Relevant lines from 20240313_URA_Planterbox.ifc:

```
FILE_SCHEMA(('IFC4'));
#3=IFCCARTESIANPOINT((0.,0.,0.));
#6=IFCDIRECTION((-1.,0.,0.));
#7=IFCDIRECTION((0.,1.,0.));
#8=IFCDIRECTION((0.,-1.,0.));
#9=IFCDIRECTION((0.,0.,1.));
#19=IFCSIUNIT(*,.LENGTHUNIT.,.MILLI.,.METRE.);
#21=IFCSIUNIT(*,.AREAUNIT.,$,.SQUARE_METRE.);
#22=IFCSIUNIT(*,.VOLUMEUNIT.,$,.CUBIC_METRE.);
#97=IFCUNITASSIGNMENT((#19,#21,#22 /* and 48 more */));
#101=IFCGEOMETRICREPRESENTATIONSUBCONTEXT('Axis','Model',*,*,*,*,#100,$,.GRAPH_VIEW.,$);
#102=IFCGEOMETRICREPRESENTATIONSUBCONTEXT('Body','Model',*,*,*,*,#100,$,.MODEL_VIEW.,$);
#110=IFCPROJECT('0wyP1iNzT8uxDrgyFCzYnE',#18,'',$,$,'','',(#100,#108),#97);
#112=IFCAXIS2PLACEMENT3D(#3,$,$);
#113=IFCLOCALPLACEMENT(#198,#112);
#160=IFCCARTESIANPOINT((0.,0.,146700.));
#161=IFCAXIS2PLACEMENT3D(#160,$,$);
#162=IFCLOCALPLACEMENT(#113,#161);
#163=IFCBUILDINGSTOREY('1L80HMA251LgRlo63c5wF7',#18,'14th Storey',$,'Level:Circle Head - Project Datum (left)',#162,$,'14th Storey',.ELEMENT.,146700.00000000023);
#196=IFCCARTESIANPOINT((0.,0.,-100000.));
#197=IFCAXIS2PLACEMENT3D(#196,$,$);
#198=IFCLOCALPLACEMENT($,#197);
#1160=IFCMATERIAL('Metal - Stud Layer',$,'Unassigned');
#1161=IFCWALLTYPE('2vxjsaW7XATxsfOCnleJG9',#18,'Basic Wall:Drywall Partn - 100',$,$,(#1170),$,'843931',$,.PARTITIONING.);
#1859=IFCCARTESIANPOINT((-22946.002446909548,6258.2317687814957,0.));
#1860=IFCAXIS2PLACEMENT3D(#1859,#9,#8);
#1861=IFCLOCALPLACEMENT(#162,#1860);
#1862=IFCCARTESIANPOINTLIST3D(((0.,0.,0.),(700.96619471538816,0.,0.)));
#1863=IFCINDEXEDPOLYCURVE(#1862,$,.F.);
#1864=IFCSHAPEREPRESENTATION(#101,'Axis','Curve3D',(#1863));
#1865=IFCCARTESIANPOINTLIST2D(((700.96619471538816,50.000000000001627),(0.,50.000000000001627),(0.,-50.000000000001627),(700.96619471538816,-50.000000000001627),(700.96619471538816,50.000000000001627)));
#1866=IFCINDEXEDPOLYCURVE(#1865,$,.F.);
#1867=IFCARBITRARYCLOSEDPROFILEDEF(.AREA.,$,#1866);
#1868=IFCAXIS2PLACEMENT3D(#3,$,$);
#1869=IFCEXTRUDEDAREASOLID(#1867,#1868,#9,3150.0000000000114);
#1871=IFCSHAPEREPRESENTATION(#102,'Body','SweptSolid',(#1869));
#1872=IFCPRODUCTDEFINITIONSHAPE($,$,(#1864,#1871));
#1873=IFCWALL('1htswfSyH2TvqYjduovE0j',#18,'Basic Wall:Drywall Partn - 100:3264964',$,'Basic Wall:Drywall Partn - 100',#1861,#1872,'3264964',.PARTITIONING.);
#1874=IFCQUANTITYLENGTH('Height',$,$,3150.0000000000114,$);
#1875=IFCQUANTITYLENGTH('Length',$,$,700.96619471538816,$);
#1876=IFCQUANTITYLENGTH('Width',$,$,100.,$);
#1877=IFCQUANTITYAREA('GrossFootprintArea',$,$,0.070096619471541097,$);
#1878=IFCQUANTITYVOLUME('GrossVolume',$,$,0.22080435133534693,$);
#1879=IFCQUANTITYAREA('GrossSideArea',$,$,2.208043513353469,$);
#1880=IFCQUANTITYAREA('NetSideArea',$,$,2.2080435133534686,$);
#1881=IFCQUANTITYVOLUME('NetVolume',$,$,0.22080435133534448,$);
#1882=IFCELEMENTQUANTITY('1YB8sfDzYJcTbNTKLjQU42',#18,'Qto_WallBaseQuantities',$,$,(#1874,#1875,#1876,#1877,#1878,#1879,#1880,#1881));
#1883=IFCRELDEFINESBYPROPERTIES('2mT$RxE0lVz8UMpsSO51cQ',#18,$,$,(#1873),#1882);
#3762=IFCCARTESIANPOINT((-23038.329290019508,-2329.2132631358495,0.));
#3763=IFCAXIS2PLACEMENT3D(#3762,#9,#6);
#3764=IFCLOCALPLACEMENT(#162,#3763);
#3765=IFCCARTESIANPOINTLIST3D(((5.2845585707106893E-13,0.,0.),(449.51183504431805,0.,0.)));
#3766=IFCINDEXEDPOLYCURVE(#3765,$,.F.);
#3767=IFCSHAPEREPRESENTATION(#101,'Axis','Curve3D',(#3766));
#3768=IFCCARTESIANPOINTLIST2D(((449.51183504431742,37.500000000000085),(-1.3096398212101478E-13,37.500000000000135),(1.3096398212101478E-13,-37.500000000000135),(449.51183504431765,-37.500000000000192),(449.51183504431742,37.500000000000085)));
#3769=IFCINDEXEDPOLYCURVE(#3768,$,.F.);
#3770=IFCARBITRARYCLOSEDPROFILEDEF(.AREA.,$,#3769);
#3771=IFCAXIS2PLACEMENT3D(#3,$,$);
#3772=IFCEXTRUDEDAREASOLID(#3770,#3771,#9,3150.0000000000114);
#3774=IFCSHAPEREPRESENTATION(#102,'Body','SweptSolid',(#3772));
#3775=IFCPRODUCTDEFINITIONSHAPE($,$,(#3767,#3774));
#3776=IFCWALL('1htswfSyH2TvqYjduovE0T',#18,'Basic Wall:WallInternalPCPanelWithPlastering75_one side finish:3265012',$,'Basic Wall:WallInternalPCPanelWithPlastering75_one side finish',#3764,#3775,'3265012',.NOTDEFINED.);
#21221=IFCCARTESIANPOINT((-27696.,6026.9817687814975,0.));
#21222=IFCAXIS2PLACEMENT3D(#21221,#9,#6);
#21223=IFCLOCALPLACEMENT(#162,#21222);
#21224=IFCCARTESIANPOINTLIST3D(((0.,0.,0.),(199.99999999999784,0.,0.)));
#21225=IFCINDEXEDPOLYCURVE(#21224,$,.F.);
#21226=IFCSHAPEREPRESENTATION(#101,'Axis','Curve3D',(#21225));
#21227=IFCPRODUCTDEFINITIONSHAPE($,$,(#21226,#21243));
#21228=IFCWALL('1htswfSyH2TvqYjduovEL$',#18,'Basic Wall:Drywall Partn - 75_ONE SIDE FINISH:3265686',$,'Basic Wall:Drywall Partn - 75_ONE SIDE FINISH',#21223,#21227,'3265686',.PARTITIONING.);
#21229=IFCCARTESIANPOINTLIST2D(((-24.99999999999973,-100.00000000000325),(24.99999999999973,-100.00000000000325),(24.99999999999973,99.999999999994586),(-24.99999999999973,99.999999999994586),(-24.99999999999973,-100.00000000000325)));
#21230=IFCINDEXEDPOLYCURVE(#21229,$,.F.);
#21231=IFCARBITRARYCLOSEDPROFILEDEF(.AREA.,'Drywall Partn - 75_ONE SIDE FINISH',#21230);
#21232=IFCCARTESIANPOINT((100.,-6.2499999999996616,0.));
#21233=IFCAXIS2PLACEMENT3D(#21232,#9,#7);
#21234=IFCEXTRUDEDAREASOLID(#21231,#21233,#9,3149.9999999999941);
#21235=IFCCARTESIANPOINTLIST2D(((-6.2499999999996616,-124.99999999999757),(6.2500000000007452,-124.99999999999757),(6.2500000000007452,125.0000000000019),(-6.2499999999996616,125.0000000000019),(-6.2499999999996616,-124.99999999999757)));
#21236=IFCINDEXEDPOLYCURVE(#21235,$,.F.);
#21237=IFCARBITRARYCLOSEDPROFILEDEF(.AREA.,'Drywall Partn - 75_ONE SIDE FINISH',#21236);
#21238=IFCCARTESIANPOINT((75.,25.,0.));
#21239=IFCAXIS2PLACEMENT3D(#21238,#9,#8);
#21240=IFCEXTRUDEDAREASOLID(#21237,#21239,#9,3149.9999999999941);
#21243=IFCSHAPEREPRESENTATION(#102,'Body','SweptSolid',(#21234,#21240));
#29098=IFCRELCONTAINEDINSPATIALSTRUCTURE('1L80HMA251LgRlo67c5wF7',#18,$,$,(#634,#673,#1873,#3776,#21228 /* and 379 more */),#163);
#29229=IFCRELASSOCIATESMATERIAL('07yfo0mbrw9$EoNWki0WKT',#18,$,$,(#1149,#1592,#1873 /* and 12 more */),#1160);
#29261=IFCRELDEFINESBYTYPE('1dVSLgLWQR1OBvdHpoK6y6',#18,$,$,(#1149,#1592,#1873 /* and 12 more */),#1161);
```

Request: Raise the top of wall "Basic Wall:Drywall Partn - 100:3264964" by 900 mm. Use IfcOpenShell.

```python
import ifcopenshell
import ifcopenshell.api.pset
import ifcopenshell.geom
import ifcopenshell.util.element
import ifcopenshell.util.representation
import ifcopenshell.util.shape
import ifcopenshell.util.unit

model = ifcopenshell.open("20240313_URA_Planterbox.ifc")
unit_scale = ifcopenshell.util.unit.calculate_unit_scale(model)
area_scale = ifcopenshell.util.unit.calculate_unit_scale(model, "AREAUNIT")
volume_scale = ifcopenshell.util.unit.calculate_unit_scale(model, "VOLUMEUNIT")
settings = ifcopenshell.geom.settings()


def volume(element):
    """Net volume in cubic metres, openings subtracted."""
    shape = ifcopenshell.geom.create_shape(settings, element)
    return ifcopenshell.util.shape.get_volume(shape.geometry)


wall = model.by_guid("1htswfSyH2TvqYjduovE0j")
before = volume(wall)

body = ifcopenshell.util.representation.get_representation(wall, "Model", "Body")
solid = body.Items[0]
old_height = solid.Depth
solid.Depth += 0.9 / unit_scale
after = volume(wall)
thickness = 0.1  # wall thickness in metres

# Update the stored height, areas and volumes.
qto = model.by_id(ifcopenshell.util.element.get_pset(wall, "Qto_WallBaseQuantities", should_inherit=False)["id"])
ifcopenshell.api.pset.edit_qto(model, qto=qto, properties={
    "Height": solid.Depth,
    "GrossVolume": ifcopenshell.util.element.get_pset(wall, "Qto_WallBaseQuantities", "GrossVolume") * solid.Depth / old_height,
    "GrossSideArea": ifcopenshell.util.element.get_pset(wall, "Qto_WallBaseQuantities", "GrossSideArea") * solid.Depth / old_height,
    "NetSideArea": after / thickness / area_scale,
    "NetVolume": after / volume_scale,
})

print(f"height {old_height:g} -> {solid.Depth:g}, volume {before:.3f} -> {after:.3f} m3")

model.write("20240313_URA_Planterbox_v2.ifc")
```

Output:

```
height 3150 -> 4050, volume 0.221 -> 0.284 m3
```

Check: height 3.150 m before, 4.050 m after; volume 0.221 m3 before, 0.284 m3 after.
